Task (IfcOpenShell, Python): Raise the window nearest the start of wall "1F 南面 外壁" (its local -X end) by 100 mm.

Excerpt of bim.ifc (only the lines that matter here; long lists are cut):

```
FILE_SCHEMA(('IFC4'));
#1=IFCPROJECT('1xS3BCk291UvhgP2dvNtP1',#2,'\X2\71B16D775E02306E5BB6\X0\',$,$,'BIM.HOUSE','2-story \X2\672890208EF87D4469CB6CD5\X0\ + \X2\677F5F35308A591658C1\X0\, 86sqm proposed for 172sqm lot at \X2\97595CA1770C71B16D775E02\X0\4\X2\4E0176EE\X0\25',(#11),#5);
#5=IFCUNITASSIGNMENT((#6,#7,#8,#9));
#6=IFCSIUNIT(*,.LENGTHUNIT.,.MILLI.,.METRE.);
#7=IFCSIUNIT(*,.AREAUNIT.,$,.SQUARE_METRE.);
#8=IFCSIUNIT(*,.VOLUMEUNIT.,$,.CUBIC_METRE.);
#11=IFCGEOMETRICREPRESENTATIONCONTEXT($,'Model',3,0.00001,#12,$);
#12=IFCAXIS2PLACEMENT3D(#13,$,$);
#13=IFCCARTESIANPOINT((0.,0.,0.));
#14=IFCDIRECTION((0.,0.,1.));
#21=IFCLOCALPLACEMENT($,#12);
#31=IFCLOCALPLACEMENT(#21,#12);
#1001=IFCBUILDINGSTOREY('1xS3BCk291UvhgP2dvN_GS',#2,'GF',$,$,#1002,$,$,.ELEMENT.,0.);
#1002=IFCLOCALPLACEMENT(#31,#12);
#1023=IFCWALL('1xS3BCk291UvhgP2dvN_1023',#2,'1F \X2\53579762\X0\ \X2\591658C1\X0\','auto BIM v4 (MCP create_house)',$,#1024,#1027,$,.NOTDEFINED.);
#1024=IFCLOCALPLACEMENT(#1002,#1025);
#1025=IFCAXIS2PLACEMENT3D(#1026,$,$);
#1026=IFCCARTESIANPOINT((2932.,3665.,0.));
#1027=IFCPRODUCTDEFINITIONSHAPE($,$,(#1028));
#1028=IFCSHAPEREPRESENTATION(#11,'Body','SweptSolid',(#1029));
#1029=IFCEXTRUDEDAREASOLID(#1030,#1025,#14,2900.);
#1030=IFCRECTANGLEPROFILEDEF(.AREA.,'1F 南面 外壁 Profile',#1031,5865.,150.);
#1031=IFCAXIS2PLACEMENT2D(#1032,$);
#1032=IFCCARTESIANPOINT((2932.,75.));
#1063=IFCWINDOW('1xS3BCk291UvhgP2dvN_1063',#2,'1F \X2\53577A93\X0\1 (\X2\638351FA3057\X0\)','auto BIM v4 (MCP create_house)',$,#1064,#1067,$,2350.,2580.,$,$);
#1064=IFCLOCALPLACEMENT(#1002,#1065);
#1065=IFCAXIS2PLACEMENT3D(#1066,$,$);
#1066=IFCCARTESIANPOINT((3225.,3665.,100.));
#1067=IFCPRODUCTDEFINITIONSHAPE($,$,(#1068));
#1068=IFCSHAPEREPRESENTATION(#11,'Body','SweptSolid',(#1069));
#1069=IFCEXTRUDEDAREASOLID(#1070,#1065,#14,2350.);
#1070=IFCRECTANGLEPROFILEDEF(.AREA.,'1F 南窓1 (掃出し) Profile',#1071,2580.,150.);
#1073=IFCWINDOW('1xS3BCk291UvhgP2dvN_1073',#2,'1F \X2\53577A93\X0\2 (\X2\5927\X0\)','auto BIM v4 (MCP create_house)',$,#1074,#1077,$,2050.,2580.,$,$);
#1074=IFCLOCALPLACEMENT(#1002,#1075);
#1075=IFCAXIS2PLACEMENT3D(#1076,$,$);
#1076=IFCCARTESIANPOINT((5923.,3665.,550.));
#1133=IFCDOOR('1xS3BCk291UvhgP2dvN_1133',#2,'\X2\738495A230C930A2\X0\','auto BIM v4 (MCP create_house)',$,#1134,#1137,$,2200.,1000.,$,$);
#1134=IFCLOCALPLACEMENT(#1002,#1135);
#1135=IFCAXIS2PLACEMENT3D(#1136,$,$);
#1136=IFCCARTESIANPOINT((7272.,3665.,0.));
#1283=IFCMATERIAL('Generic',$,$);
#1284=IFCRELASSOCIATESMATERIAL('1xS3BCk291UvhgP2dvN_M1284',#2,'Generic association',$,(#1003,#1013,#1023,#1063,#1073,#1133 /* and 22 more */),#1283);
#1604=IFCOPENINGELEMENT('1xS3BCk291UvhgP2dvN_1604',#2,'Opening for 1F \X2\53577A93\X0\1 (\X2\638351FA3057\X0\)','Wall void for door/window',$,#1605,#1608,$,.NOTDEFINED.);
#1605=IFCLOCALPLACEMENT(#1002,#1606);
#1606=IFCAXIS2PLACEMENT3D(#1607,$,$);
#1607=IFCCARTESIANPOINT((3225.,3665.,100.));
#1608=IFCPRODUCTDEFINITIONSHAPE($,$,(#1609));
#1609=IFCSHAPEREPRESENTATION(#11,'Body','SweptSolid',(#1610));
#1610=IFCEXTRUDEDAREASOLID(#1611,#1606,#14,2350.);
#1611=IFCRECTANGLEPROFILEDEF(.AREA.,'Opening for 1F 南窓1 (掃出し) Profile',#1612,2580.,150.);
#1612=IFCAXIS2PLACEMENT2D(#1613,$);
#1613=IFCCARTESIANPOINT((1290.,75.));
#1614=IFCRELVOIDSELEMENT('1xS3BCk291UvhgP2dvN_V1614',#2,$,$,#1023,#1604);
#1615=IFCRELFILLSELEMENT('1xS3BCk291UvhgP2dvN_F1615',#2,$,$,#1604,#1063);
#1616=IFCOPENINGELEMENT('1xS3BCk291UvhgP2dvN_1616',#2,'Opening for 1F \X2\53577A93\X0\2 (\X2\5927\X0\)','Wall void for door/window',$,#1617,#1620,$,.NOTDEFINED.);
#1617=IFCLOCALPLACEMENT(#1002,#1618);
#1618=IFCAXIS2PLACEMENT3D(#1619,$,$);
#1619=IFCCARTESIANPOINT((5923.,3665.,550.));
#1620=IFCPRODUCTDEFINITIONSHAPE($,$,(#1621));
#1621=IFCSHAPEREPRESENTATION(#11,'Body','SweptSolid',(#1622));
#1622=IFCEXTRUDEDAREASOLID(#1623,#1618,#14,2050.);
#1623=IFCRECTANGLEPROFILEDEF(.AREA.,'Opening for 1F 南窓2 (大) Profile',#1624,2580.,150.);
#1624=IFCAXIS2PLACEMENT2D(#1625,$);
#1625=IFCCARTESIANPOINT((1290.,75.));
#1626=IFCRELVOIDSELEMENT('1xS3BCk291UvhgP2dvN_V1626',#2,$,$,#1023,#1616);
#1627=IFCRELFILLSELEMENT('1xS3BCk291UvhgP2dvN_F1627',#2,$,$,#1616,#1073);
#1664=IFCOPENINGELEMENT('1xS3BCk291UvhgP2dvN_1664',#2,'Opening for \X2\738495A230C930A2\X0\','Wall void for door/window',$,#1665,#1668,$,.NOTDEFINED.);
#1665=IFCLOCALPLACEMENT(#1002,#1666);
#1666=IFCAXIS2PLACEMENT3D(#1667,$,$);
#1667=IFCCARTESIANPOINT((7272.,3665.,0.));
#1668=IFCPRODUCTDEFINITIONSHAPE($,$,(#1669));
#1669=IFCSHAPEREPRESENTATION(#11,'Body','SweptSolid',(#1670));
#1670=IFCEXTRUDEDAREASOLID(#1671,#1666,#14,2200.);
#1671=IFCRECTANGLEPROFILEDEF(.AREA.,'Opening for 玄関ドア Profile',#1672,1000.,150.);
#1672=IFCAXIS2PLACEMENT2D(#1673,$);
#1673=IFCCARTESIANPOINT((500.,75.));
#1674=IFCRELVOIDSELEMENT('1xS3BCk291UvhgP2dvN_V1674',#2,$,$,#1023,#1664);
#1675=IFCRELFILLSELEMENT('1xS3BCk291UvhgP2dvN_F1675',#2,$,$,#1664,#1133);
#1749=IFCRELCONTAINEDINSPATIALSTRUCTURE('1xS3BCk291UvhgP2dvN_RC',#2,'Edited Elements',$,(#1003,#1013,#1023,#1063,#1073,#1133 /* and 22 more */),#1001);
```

```python
import numpy as np
import ifcopenshell
import ifcopenshell.api.geometry
import ifcopenshell.util.placement
import ifcopenshell.util.unit

model = ifcopenshell.open("bim.ifc")
unit_scale = ifcopenshell.util.unit.calculate_unit_scale(model)

window = model.by_guid("1xS3BCk291UvhgP2dvN_1063")
opening = window.FillsVoids[0].RelatingOpeningElement
dz = 100.0

shift = np.array([0.0, 0.0, dz])
# The window is not placed relative to its opening, so move both.
for product in (opening, window):
    matrix = ifcopenshell.util.placement.get_local_placement(product.ObjectPlacement)
    matrix[:3, 3] += shift
    ifcopenshell.api.geometry.edit_object_placement(model, product=product, matrix=matrix, is_si=False)

print(f"moved by {dz * unit_scale:+.3f} m")

model.write("bim_edited.ifc")
```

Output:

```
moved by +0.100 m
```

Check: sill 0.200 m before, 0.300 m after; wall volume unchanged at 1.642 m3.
